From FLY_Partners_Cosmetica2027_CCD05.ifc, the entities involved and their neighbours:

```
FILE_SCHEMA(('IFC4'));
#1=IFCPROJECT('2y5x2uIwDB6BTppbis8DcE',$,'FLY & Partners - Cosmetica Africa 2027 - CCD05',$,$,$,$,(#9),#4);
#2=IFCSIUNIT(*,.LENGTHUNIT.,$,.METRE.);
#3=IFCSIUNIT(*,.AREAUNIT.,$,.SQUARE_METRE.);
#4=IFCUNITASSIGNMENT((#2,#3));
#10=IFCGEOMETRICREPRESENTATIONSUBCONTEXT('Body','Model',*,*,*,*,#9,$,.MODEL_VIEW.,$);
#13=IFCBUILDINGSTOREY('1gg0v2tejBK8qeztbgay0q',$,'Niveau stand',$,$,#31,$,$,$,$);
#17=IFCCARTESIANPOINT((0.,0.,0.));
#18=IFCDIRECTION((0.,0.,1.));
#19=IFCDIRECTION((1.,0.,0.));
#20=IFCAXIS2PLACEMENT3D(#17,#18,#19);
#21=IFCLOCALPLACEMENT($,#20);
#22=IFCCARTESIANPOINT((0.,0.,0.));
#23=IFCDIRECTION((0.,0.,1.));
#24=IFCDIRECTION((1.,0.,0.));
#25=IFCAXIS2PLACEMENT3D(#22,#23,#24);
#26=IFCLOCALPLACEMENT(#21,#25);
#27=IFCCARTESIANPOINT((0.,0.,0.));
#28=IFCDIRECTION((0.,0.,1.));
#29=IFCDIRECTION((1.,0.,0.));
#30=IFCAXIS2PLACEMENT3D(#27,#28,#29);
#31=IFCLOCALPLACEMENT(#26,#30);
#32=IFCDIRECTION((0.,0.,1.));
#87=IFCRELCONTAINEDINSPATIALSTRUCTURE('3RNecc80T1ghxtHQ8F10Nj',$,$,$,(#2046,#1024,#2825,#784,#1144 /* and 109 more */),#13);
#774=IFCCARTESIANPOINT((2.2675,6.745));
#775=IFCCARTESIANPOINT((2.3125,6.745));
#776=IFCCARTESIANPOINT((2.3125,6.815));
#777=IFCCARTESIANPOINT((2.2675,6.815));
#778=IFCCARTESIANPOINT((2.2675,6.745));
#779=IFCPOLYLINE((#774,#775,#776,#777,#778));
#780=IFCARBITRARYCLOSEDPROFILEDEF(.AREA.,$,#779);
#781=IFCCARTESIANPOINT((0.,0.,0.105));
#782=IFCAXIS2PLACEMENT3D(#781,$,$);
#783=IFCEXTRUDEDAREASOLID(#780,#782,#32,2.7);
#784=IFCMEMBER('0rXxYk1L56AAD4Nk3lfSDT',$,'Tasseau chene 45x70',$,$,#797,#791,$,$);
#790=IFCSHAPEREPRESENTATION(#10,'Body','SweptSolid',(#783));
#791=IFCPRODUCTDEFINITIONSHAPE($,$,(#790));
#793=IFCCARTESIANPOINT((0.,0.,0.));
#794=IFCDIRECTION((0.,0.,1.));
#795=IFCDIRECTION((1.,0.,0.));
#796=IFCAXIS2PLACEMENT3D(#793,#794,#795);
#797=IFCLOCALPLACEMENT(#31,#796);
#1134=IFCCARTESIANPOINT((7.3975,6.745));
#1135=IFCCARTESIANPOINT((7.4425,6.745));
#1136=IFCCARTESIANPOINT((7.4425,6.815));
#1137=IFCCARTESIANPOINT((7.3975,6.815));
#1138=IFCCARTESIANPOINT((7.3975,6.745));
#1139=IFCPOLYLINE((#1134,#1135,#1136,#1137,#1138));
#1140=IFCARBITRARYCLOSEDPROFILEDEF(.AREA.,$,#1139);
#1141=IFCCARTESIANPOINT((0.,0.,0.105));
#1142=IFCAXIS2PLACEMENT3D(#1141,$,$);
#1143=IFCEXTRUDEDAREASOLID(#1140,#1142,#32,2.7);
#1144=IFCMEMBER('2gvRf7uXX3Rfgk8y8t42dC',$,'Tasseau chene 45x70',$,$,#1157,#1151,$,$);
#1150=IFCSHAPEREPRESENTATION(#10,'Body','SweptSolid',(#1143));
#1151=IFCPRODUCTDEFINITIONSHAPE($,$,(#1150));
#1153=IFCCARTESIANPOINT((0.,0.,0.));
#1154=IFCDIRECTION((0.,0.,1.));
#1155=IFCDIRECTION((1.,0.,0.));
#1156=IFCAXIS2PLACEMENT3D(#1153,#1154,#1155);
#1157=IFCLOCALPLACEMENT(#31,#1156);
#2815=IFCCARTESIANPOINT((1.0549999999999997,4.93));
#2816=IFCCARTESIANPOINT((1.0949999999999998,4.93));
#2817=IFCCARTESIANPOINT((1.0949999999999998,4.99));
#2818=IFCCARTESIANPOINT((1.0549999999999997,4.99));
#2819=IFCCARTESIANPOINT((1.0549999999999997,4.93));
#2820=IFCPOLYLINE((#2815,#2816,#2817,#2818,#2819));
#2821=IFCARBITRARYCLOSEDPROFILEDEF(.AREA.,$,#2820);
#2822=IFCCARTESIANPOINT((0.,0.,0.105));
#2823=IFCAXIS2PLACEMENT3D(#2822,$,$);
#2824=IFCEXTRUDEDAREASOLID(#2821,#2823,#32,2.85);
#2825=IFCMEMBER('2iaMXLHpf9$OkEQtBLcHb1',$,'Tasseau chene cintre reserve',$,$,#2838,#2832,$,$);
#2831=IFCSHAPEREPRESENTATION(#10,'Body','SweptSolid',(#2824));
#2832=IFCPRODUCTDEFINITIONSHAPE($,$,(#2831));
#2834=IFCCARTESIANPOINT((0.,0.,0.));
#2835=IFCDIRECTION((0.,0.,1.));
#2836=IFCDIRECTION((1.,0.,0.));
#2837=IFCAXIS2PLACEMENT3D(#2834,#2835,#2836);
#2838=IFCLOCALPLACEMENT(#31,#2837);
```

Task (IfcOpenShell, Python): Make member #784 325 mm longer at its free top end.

```python
import ifcopenshell
import ifcopenshell.util.representation

model = ifcopenshell.open("FLY_Partners_Cosmetica2027_CCD05.ifc")

member = model.by_guid("0rXxYk1L56AAD4Nk3lfSDT")
change = 0.325

# The extrusion runs towards the end named, so only its depth changes.
body = ifcopenshell.util.representation.get_representation(member, "Model", "Body")
solid = body.Items[0]
old_length = solid.Depth
solid.Depth += change

print(f"length {old_length:g} -> {solid.Depth:g}")

model.write("FLY_Partners_Cosmetica2027_CCD05_v2.ifc")
```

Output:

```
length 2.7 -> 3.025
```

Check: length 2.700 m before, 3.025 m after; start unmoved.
